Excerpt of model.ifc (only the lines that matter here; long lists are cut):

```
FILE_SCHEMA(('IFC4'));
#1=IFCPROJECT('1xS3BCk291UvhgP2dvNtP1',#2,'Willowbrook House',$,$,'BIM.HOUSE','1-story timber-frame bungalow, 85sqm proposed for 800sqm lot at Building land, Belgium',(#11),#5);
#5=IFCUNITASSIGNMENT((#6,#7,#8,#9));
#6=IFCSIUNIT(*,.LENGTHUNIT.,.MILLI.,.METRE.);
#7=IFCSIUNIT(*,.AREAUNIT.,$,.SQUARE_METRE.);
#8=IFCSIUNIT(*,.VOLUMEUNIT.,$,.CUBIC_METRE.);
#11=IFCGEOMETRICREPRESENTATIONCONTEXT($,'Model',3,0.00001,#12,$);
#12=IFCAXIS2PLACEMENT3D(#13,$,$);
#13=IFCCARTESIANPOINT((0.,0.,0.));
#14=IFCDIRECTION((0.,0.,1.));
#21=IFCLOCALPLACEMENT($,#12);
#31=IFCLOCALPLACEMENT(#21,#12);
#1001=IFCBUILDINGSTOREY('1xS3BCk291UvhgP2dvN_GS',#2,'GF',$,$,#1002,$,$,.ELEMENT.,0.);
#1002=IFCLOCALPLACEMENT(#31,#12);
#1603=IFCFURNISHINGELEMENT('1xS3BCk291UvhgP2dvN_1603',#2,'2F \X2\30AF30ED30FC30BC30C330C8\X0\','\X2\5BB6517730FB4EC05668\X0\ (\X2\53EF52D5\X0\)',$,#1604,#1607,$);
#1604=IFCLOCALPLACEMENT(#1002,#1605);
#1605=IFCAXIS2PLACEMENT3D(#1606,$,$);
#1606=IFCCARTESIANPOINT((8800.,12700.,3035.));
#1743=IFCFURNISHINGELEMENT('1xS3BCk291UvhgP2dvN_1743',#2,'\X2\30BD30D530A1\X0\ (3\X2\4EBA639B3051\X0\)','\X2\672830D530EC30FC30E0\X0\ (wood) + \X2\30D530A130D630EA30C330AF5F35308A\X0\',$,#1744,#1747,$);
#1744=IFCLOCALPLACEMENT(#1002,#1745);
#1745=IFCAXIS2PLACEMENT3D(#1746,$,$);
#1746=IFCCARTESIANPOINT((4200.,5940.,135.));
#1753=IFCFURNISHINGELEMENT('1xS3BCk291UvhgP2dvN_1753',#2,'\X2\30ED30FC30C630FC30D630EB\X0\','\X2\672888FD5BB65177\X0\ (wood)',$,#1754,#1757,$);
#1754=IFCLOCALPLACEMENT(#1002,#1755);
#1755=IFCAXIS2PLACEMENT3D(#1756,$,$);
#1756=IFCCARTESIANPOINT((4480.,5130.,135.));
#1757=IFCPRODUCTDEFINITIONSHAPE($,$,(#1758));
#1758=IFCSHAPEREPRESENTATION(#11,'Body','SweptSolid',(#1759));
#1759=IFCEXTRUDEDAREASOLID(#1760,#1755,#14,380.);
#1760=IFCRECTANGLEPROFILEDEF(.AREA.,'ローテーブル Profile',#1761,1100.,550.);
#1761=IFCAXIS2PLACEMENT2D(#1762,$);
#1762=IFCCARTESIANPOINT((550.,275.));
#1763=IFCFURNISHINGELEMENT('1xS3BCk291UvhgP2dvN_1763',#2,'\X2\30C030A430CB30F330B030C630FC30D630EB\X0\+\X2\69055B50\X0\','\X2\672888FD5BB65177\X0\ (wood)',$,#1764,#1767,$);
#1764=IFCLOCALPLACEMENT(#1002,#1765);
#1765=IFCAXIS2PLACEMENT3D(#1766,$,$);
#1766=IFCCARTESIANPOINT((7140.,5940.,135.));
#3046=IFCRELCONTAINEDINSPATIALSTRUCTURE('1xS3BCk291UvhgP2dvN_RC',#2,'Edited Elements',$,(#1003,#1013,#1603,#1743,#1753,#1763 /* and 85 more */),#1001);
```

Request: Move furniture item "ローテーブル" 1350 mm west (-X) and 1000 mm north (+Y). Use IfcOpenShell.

```python
import ifcopenshell
import ifcopenshell.api.geometry
import ifcopenshell.util.placement

model = ifcopenshell.open("model.ifc")

item = model.by_guid("1xS3BCk291UvhgP2dvN_1753")
matrix = ifcopenshell.util.placement.get_local_placement(item.ObjectPlacement)
matrix[0, 3] -= 1350.0
matrix[1, 3] += 1000.0
ifcopenshell.api.geometry.edit_object_placement(model, product=item, matrix=matrix, is_si=False)

print(ifcopenshell.util.placement.get_local_placement(item.ObjectPlacement).round(3) + 0.0)

model.write("model-out.ifc")
```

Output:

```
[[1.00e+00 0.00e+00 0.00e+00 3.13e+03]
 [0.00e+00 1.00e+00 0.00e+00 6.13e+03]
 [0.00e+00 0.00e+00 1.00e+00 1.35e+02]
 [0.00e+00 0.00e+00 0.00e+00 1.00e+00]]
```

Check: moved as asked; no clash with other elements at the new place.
